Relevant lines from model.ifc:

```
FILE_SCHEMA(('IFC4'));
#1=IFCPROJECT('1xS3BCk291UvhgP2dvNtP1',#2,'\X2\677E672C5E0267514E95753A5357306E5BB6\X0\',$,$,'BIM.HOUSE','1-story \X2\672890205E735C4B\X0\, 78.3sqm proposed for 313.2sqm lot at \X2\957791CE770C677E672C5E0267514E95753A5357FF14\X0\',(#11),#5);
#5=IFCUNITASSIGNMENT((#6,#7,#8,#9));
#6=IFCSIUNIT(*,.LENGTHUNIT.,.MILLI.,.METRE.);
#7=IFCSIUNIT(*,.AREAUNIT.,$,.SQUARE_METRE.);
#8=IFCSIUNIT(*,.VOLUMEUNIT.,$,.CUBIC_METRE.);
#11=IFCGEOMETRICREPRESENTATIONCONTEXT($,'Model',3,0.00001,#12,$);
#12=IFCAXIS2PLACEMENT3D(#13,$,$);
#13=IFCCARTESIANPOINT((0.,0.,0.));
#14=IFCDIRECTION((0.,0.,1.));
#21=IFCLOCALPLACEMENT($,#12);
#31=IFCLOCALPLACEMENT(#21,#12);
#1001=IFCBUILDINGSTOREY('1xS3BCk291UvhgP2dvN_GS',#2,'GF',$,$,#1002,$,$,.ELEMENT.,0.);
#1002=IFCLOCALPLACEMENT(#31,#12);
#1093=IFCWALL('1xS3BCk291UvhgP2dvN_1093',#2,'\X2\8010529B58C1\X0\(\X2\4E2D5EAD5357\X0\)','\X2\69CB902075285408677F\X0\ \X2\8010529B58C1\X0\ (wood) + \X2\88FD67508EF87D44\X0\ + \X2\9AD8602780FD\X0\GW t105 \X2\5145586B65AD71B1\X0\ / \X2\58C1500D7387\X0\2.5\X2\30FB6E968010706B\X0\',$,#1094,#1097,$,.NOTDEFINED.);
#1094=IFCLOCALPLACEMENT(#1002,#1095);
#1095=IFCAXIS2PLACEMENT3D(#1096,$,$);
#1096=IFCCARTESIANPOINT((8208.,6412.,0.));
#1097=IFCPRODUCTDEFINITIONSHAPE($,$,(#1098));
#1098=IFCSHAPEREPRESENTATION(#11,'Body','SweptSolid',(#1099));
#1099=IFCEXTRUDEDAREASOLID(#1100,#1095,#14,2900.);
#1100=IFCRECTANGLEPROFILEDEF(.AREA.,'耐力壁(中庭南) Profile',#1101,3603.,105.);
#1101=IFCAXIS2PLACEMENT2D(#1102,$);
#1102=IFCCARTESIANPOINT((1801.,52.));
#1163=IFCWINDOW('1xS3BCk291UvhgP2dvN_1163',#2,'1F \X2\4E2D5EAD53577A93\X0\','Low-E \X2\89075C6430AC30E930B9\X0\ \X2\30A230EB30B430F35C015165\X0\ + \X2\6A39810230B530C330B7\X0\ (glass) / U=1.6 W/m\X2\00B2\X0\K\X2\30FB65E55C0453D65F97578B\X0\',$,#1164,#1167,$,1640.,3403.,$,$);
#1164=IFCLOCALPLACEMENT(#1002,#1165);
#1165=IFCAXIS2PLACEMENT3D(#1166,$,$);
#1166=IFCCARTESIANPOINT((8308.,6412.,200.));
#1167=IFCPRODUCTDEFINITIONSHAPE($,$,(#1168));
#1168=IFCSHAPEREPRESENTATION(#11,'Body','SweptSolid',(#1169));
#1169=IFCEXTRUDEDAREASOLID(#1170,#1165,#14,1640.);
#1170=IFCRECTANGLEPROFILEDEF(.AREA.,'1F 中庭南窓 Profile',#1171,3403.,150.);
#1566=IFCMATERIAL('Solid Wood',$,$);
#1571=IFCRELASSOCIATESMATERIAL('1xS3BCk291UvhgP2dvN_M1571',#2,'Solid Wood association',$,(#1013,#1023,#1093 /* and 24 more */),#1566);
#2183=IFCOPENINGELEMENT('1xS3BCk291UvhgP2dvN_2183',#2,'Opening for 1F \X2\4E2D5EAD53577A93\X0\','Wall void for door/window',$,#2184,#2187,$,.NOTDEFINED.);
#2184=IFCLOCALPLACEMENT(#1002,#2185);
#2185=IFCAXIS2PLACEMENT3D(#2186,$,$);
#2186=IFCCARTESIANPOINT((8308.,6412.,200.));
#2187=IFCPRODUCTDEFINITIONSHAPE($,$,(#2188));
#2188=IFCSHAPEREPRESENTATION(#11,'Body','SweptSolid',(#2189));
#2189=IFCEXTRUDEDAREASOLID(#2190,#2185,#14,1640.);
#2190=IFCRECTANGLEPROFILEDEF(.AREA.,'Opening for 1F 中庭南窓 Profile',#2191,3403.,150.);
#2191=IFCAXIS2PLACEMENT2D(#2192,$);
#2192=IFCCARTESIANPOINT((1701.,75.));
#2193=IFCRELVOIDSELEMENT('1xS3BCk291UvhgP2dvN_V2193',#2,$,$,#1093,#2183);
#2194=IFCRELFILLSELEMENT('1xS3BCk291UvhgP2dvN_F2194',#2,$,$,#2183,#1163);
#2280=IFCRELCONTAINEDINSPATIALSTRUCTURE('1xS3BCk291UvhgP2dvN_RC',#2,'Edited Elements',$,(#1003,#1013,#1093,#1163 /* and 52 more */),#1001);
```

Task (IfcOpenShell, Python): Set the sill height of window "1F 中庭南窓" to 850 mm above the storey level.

```python
import numpy as np
import ifcopenshell
import ifcopenshell.api.geometry
import ifcopenshell.geom
import ifcopenshell.util.element
import ifcopenshell.util.placement
import ifcopenshell.util.shape
import ifcopenshell.util.unit

model = ifcopenshell.open("model.ifc")
unit_scale = ifcopenshell.util.unit.calculate_unit_scale(model)

window = model.by_id(1163)
opening = window.FillsVoids[0].RelatingOpeningElement
storey = ifcopenshell.util.element.get_container(window, ifc_class="IfcBuildingStorey")
level = ifcopenshell.util.placement.get_local_placement(storey.ObjectPlacement)[2, 3]

# The opening's origin need not be at the sill, so measure its lowest point.
shape = ifcopenshell.geom.create_shape(ifcopenshell.geom.settings(), opening)
bottom = ifcopenshell.util.shape.get_shape_bottom_elevation(shape, shape.geometry) / unit_scale
dz = level + 0.85 / unit_scale - bottom

shift = np.array([0.0, 0.0, dz])
# The window is not placed relative to its opening, so move both.
for product in (opening, window):
    matrix = ifcopenshell.util.placement.get_local_placement(product.ObjectPlacement)
    matrix[:3, 3] += shift
    ifcopenshell.api.geometry.edit_object_placement(model, product=product, matrix=matrix, is_si=False)

print(f"moved by {dz * unit_scale:+.3f} m")

model.write("model-out.ifc")
```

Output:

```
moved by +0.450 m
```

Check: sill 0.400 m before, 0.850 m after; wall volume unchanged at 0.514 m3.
